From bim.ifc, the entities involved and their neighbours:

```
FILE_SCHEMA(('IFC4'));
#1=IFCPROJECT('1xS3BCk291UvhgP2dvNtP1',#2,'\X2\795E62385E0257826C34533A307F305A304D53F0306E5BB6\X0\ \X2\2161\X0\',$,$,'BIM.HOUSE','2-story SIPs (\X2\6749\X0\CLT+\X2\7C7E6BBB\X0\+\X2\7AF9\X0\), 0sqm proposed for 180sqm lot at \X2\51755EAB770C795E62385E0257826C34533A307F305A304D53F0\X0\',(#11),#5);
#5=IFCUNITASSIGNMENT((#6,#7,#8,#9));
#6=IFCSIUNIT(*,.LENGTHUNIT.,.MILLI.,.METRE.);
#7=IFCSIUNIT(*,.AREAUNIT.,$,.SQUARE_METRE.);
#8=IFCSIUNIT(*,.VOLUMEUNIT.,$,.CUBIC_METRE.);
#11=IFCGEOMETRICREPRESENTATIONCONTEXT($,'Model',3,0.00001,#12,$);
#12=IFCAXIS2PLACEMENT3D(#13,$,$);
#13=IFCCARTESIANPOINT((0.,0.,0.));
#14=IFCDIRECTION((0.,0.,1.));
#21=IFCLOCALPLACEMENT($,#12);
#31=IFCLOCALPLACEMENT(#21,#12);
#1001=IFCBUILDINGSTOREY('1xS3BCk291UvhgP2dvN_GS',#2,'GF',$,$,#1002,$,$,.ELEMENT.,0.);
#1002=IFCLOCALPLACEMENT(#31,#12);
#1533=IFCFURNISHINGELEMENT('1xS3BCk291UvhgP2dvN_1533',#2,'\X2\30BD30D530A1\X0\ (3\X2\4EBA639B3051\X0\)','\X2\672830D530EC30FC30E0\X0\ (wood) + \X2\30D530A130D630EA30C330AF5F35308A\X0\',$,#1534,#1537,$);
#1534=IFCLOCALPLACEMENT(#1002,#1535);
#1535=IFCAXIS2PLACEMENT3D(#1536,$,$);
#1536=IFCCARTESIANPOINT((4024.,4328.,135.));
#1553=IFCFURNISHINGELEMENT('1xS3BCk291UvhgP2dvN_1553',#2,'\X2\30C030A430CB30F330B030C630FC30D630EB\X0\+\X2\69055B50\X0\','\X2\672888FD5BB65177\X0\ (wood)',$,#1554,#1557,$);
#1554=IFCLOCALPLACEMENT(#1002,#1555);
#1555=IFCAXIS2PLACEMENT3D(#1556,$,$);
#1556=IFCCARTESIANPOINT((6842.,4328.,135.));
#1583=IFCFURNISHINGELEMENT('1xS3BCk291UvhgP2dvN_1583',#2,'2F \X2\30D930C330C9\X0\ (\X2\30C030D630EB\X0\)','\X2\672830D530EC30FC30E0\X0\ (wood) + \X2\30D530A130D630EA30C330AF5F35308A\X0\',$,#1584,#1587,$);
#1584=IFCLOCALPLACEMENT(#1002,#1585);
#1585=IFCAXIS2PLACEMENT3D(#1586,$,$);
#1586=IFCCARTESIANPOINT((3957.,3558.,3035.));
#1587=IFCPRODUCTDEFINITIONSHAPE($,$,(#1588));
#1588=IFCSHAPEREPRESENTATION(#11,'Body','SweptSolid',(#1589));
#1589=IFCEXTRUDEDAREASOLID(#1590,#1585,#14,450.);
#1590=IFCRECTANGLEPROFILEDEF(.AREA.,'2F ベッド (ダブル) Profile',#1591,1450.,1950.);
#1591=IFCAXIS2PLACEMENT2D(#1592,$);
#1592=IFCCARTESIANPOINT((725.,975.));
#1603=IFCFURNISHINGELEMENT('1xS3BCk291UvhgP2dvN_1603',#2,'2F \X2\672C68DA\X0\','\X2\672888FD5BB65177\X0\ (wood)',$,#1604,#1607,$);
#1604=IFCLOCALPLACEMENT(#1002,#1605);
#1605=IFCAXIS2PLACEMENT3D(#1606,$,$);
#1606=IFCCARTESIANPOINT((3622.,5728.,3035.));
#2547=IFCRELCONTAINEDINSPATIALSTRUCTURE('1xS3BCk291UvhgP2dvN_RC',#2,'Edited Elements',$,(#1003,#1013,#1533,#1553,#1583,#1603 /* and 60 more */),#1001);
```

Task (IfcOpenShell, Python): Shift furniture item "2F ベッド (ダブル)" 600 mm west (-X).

```python
import ifcopenshell
import ifcopenshell.api.geometry
import ifcopenshell.util.placement

model = ifcopenshell.open("bim.ifc")

item = model.by_id(1583)
matrix = ifcopenshell.util.placement.get_local_placement(item.ObjectPlacement)
matrix[0, 3] -= 600.0
ifcopenshell.api.geometry.edit_object_placement(model, product=item, matrix=matrix, is_si=False)

print(ifcopenshell.util.placement.get_local_placement(item.ObjectPlacement).round(3) + 0.0)

model.write("bim-out.ifc")
```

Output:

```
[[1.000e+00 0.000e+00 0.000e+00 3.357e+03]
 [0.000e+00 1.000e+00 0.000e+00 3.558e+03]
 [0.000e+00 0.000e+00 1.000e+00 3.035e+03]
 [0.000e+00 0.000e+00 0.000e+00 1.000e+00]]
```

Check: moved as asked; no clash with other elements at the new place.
